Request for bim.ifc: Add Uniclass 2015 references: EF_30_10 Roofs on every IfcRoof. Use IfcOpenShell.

First a look at what the model holds.

```python
import ifcopenshell

model = ifcopenshell.open("bim.ifc")
print(model.schema)
print("classifications:", [c.Name for c in model.by_type("IfcClassification")])
for ifc_class in ("IfcDoor", "IfcRoof", "IfcStair", "IfcWall", "IfcWindow"):
    print(ifc_class, len(model.by_type(ifc_class)))
```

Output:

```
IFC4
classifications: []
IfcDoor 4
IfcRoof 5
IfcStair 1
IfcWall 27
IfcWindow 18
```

```python
import ifcopenshell
import ifcopenshell.api.classification

model = ifcopenshell.open("bim.ifc")

system = ifcopenshell.api.classification.add_classification(model, classification="Uniclass 2015")

codes = {
    "IfcRoof": ("EF_30_10", "Roofs"),
}
for ifc_class, (code, name) in codes.items():
    products = model.by_type(ifc_class)
    ifcopenshell.api.classification.add_reference(
        model, products=products, classification=system, identification=code, name=name
    )
    print(code, len(products))

model.write("bim_rev.ifc")
```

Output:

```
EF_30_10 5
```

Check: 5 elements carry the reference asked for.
